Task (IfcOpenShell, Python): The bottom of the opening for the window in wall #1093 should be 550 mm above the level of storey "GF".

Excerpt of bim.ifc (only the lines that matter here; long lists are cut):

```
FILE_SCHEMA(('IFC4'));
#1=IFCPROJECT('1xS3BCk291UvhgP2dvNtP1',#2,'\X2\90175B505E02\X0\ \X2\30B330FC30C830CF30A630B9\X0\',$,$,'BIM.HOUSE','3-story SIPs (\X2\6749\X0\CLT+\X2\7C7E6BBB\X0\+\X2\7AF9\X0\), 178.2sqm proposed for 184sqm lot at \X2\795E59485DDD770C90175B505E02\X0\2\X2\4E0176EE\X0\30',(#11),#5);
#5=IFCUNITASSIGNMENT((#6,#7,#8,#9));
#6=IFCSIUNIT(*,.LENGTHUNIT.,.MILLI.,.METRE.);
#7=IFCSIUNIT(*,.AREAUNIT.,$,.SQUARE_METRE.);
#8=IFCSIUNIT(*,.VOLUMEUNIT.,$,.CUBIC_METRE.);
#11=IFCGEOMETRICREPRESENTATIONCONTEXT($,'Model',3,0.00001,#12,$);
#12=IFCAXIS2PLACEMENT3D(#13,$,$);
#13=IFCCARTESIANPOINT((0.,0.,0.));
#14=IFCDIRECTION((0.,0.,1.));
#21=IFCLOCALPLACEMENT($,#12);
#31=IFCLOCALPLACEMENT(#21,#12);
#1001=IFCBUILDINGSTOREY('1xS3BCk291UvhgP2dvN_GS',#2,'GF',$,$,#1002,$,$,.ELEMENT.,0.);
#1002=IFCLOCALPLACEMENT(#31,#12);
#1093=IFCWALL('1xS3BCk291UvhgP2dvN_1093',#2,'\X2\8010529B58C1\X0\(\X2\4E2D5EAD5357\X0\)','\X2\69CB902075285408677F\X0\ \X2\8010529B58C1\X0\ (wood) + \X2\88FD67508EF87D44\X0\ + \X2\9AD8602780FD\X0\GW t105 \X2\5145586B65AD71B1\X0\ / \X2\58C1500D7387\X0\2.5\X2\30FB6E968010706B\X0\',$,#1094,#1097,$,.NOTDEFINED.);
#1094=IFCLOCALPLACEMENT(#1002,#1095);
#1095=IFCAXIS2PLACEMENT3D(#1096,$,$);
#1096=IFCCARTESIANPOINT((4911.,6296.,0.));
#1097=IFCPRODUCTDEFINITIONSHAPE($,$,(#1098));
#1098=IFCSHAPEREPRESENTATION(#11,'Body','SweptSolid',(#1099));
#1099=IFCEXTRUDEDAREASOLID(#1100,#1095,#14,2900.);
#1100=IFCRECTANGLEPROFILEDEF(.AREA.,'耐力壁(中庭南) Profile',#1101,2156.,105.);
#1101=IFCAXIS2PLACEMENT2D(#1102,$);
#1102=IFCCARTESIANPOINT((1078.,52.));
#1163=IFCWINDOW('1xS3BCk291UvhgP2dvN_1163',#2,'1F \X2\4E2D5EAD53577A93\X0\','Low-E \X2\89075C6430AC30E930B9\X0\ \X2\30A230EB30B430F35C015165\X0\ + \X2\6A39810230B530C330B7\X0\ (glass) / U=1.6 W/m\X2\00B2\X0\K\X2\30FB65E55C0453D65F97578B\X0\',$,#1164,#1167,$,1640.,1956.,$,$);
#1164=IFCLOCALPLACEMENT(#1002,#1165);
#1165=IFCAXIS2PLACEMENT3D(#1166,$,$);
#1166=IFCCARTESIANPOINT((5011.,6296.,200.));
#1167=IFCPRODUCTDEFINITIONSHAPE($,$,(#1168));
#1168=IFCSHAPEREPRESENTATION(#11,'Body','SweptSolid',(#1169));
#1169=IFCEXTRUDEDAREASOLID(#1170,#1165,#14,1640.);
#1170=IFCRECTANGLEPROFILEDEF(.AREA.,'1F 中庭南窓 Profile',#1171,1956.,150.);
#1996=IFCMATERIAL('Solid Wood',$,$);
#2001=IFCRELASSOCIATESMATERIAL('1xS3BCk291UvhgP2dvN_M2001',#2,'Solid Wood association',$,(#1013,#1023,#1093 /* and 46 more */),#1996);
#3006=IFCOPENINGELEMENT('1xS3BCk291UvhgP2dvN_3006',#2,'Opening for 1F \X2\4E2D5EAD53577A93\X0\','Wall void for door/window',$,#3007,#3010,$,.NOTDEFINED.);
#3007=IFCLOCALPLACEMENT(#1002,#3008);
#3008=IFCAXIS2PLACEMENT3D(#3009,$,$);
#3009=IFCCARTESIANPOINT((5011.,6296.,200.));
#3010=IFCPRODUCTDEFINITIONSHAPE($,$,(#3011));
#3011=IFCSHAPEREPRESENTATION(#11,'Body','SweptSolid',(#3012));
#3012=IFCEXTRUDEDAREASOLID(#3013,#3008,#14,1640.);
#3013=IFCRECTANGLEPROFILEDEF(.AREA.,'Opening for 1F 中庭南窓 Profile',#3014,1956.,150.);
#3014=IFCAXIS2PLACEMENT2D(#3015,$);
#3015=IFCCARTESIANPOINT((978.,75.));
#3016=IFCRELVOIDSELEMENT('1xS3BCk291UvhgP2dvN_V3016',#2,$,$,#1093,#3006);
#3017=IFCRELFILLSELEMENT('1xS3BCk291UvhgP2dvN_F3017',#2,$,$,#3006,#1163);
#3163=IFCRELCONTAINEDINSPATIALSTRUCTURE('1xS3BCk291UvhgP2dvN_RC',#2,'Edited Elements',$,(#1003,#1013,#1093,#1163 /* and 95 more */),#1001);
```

```python
import numpy as np
import ifcopenshell
import ifcopenshell.api.geometry
import ifcopenshell.geom
import ifcopenshell.util.element
import ifcopenshell.util.placement
import ifcopenshell.util.shape
import ifcopenshell.util.unit

model = ifcopenshell.open("bim.ifc")
unit_scale = ifcopenshell.util.unit.calculate_unit_scale(model)

window = model.by_id(1163)
opening = window.FillsVoids[0].RelatingOpeningElement
storey = ifcopenshell.util.element.get_container(window, ifc_class="IfcBuildingStorey")
level = ifcopenshell.util.placement.get_local_placement(storey.ObjectPlacement)[2, 3]

# The opening's origin need not be at the sill, so measure its lowest point.
shape = ifcopenshell.geom.create_shape(ifcopenshell.geom.settings(), opening)
bottom = ifcopenshell.util.shape.get_shape_bottom_elevation(shape, shape.geometry) / unit_scale
dz = level + 550.0 - bottom

shift = np.array([0.0, 0.0, dz])
# The window is not placed relative to its opening, so move both.
for product in (opening, window):
    matrix = ifcopenshell.util.placement.get_local_placement(product.ObjectPlacement)
    matrix[:3, 3] += shift
    ifcopenshell.api.geometry.edit_object_placement(model, product=product, matrix=matrix, is_si=False)

print(f"moved by {dz * unit_scale:+.3f} m")

model.write("bim_edited.ifc")
```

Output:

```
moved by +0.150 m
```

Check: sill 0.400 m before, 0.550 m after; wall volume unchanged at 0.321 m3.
